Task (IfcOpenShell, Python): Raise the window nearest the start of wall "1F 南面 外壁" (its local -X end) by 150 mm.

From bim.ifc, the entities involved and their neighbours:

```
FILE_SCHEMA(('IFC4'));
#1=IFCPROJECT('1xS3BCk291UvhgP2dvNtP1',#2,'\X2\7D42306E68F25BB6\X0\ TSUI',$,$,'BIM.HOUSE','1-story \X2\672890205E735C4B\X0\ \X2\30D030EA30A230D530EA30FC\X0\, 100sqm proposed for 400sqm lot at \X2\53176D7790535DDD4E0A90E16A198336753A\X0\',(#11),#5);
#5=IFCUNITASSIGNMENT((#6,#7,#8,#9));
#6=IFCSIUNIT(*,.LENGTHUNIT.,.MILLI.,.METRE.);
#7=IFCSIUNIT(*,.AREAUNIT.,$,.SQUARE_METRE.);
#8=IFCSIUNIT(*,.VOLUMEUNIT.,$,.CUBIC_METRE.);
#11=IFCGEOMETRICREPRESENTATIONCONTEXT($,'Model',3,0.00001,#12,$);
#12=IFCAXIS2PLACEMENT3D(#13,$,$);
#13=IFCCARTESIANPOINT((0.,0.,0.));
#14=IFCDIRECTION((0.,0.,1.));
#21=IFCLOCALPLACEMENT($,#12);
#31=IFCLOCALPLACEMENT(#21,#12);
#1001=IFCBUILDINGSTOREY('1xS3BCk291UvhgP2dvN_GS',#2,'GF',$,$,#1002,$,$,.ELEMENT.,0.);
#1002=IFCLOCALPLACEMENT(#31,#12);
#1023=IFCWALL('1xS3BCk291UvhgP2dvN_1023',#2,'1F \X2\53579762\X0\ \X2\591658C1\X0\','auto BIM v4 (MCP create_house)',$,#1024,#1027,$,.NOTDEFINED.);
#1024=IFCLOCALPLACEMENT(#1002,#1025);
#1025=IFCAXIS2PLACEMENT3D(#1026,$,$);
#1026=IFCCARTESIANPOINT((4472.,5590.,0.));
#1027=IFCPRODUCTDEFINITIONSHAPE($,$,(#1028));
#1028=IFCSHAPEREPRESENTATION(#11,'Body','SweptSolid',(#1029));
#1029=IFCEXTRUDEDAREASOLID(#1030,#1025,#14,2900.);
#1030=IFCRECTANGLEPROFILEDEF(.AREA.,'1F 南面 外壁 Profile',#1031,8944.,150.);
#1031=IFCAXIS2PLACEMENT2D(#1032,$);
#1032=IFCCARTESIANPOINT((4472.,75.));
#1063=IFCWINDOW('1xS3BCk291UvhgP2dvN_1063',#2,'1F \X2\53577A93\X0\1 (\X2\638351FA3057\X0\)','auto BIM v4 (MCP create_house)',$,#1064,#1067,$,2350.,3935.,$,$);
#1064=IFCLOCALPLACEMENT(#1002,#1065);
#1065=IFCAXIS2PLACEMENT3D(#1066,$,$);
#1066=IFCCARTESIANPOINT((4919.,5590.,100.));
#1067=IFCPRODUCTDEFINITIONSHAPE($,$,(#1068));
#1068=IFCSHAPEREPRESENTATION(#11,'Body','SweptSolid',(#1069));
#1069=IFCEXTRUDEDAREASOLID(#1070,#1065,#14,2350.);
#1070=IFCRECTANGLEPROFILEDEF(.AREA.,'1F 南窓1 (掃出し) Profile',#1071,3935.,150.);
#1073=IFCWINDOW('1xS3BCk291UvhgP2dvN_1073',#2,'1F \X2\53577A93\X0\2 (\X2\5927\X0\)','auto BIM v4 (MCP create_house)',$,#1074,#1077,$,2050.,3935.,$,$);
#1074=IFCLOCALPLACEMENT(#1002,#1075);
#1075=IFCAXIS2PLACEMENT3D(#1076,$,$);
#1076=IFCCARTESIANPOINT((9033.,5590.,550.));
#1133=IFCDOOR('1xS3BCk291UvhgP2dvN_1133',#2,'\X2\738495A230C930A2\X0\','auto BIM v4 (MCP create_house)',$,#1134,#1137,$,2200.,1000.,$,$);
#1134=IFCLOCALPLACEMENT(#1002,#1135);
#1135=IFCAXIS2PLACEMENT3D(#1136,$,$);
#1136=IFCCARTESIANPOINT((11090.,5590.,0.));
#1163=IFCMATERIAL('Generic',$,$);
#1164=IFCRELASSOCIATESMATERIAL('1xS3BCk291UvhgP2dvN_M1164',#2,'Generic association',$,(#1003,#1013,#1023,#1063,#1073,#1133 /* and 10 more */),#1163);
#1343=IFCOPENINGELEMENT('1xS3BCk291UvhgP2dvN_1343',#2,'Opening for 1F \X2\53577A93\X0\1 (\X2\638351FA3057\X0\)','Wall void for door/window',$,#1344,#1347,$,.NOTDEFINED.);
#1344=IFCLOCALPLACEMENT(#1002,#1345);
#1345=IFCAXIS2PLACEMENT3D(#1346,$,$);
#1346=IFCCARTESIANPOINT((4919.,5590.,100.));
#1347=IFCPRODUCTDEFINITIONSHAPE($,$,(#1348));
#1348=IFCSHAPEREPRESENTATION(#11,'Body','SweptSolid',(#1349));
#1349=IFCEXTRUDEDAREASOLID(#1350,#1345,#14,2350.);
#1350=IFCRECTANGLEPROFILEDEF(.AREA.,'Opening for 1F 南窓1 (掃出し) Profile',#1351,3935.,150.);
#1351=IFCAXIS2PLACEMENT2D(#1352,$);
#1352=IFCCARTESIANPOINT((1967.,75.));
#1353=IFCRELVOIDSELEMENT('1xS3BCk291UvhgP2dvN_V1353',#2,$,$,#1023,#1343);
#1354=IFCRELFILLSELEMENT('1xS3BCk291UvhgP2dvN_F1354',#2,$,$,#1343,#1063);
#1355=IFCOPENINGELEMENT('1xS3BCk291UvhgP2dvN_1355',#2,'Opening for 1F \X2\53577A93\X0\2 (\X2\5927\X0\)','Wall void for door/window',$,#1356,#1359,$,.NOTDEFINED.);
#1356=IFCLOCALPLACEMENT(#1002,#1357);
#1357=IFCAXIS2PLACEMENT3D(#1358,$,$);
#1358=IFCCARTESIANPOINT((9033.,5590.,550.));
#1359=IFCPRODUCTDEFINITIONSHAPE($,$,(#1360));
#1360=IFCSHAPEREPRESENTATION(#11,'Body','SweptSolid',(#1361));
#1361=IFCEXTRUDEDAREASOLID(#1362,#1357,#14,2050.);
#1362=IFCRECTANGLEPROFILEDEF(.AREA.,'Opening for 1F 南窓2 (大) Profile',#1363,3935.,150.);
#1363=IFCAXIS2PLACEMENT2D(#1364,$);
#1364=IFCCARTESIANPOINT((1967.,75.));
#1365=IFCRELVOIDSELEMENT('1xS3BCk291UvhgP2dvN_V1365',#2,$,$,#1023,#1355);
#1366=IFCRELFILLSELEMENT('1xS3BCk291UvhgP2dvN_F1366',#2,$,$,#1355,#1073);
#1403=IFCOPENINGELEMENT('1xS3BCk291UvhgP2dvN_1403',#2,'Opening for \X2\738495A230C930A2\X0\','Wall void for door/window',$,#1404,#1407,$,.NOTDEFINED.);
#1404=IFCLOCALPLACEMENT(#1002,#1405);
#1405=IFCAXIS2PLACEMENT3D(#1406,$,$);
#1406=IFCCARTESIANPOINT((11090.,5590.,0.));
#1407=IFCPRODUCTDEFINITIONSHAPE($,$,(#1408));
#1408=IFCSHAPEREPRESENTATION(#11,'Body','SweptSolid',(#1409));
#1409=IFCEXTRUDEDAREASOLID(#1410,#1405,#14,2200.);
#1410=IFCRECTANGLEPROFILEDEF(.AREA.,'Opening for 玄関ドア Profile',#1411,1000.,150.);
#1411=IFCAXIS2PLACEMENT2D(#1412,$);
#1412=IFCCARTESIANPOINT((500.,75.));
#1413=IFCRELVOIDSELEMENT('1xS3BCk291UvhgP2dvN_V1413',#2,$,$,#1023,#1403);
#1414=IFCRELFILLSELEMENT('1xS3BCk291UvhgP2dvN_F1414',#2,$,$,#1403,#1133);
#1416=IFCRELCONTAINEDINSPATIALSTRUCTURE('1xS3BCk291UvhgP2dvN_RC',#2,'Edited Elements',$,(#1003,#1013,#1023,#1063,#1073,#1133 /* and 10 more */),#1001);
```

```python
import numpy as np
import ifcopenshell
import ifcopenshell.api.geometry
import ifcopenshell.util.placement
import ifcopenshell.util.unit

model = ifcopenshell.open("bim.ifc")
unit_scale = ifcopenshell.util.unit.calculate_unit_scale(model)

window = model.by_guid("1xS3BCk291UvhgP2dvN_1063")
opening = window.FillsVoids[0].RelatingOpeningElement
dz = 150.0

shift = np.array([0.0, 0.0, dz])
# The window is not placed relative to its opening, so move both.
for product in (opening, window):
    matrix = ifcopenshell.util.placement.get_local_placement(product.ObjectPlacement)
    matrix[:3, 3] += shift
    ifcopenshell.api.geometry.edit_object_placement(model, product=product, matrix=matrix, is_si=False)

print(f"moved by {dz * unit_scale:+.3f} m")

model.write("bim_rev.ifc")
```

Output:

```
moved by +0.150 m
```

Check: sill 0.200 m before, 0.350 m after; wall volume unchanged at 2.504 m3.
